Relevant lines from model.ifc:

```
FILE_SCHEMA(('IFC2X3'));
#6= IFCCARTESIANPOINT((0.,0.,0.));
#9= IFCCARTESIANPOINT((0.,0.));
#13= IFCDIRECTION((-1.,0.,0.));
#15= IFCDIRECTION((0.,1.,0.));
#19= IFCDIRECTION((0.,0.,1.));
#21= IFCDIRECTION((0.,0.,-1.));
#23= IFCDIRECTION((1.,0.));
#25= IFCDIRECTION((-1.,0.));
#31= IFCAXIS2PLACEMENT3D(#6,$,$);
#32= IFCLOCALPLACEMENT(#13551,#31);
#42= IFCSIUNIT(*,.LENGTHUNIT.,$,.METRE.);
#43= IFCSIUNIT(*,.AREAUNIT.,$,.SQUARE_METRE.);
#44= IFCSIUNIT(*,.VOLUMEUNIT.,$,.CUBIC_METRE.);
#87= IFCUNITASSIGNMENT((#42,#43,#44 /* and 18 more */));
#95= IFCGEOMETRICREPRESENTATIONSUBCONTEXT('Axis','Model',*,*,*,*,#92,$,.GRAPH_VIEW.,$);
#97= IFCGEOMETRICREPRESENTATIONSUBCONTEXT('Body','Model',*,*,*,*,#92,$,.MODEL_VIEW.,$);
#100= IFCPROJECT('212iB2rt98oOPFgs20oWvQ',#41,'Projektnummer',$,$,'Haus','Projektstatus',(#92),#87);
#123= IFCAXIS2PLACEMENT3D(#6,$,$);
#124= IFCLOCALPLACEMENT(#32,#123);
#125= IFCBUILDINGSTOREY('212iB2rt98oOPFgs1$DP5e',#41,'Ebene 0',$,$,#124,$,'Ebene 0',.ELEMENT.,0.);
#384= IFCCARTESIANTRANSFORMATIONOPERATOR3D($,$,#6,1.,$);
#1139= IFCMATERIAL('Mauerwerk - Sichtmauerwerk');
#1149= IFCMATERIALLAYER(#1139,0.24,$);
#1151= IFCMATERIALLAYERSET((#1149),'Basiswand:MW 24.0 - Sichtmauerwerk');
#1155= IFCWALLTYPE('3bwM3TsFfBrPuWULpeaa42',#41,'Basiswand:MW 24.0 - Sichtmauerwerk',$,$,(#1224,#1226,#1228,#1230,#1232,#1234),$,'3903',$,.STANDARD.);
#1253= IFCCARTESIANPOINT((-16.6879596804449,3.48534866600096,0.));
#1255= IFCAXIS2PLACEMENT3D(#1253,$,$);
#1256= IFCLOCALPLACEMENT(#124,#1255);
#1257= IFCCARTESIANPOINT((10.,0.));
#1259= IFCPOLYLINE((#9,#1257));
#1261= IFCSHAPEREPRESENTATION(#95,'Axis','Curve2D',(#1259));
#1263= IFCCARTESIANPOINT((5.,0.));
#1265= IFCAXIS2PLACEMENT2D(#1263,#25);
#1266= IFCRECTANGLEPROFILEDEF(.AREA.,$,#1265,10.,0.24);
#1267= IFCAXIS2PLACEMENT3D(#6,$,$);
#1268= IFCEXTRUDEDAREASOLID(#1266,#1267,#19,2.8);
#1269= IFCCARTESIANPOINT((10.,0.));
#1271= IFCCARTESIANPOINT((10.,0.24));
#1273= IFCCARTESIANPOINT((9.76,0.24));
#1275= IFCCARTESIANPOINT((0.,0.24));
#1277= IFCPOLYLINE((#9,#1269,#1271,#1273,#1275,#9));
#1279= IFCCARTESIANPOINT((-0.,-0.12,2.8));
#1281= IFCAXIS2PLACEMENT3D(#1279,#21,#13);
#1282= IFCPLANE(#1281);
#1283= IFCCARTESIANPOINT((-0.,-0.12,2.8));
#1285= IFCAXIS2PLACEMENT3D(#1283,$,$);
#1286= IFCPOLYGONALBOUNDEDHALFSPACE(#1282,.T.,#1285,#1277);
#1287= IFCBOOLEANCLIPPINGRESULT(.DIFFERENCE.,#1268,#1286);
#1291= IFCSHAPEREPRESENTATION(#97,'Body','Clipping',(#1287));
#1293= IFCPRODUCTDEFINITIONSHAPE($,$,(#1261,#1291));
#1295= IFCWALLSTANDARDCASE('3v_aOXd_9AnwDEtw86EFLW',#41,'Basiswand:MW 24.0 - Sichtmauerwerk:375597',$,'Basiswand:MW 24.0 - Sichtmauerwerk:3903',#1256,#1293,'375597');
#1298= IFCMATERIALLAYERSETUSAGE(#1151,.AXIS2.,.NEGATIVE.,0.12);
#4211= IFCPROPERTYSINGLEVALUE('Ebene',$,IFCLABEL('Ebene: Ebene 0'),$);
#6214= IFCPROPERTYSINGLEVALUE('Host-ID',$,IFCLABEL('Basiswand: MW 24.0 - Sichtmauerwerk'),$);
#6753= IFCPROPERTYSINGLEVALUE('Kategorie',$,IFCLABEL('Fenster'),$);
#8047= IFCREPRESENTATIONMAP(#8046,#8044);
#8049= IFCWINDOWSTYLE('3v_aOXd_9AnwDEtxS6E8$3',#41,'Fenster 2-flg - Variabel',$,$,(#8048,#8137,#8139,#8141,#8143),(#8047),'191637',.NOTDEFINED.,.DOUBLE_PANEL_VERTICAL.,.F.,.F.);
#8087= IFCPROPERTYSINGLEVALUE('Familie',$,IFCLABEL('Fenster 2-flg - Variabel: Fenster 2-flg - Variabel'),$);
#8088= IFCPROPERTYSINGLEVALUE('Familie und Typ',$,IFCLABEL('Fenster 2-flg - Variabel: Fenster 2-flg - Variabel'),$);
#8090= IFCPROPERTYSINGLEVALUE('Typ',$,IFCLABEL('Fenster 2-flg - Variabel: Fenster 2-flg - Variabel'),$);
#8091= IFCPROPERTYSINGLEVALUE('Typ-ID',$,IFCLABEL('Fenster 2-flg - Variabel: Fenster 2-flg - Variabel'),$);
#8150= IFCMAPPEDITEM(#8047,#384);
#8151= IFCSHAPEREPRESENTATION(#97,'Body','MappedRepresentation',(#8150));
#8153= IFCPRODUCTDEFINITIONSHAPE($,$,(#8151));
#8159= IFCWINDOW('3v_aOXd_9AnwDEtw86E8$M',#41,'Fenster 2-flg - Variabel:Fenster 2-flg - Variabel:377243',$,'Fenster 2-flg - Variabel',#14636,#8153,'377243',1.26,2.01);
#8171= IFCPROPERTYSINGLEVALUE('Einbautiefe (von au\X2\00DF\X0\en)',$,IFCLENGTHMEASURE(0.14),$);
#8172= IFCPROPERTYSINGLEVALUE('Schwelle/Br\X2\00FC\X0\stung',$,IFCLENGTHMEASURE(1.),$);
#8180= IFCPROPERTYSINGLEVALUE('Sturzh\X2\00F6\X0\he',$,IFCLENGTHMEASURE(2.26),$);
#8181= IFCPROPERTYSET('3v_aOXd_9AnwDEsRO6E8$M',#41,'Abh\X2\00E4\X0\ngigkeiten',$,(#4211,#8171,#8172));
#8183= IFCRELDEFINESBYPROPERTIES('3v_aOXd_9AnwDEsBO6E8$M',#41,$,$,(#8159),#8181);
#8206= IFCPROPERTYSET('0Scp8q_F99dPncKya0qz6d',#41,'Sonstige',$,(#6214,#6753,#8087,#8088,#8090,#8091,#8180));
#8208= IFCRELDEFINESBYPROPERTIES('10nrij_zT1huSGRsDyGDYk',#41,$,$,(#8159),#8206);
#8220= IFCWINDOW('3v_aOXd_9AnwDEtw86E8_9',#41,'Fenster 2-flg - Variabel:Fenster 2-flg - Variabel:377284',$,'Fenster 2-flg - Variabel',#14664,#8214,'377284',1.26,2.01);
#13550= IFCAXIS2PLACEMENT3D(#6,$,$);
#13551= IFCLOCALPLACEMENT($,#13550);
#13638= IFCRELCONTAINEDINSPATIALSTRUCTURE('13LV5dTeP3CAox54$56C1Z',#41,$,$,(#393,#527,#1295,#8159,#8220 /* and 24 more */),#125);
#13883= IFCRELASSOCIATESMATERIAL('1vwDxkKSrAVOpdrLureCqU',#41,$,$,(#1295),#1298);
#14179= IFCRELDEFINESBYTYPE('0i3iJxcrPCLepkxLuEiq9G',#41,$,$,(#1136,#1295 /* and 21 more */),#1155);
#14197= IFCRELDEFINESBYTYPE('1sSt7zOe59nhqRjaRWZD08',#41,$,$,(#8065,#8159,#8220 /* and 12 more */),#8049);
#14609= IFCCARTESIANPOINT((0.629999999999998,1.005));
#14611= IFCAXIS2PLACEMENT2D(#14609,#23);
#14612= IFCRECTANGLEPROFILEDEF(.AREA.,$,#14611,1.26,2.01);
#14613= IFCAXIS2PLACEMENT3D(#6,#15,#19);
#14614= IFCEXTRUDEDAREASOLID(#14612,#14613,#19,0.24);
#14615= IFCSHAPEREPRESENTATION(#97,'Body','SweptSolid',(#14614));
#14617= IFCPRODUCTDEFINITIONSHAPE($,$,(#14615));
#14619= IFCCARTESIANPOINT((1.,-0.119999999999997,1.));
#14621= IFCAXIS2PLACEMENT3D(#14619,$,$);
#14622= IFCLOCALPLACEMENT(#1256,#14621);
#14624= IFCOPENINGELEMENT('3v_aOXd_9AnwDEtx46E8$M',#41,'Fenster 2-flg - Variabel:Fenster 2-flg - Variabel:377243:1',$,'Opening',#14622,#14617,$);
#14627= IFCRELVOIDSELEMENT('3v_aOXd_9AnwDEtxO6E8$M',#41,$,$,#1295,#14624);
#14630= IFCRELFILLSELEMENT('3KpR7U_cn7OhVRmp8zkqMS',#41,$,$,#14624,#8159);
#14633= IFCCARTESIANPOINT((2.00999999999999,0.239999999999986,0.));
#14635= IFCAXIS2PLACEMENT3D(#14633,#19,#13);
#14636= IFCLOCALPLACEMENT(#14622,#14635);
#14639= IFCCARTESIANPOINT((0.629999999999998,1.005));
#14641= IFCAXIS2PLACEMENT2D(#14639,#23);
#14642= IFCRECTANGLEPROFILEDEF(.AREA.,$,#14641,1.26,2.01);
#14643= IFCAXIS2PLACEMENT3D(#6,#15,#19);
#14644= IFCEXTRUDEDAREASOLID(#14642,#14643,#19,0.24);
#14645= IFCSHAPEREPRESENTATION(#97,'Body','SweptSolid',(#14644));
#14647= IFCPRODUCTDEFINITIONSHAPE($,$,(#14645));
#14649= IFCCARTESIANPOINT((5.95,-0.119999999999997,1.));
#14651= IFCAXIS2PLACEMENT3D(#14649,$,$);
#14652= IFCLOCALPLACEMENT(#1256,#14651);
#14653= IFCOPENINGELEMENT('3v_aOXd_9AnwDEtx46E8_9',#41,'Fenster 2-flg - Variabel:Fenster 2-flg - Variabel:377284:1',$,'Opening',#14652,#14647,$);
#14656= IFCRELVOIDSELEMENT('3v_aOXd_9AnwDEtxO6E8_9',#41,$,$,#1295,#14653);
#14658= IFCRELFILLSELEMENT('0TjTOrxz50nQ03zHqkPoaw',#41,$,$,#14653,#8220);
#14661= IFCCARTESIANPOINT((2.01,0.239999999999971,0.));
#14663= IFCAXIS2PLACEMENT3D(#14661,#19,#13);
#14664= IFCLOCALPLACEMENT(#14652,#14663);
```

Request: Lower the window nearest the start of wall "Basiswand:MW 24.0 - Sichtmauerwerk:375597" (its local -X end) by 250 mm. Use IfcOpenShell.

```python
import numpy as np
import ifcopenshell
import ifcopenshell.api.geometry
import ifcopenshell.api.pset
import ifcopenshell.util.element
import ifcopenshell.util.placement
import ifcopenshell.util.unit

model = ifcopenshell.open("model.ifc")
unit_scale = ifcopenshell.util.unit.calculate_unit_scale(model)

window = model.by_guid("3v_aOXd_9AnwDEtw86E8$M")
opening = window.FillsVoids[0].RelatingOpeningElement
dz = -0.25 / unit_scale

shift = np.array([0.0, 0.0, dz])
# The window is placed relative to its opening, so it follows when the opening moves.
matrix = ifcopenshell.util.placement.get_local_placement(opening.ObjectPlacement)
matrix[:3, 3] += shift
ifcopenshell.api.geometry.edit_object_placement(
    model, product=opening, matrix=matrix, is_si=False, should_transform_children=True
)

# Keep the stored heights in step.
pset = model.by_id(ifcopenshell.util.element.get_pset(window, "Abhängigkeiten", should_inherit=False)["id"])
ifcopenshell.api.pset.edit_pset(model, pset=pset, properties={
    "Schwelle/Brüstung": model.create_entity("IfcLengthMeasure", ifcopenshell.util.element.get_pset(window, "Abhängigkeiten", "Schwelle/Brüstung") + dz),
})
pset = model.by_id(ifcopenshell.util.element.get_pset(window, "Sonstige", should_inherit=False)["id"])
ifcopenshell.api.pset.edit_pset(model, pset=pset, properties={
    "Sturzhöhe": model.create_entity("IfcLengthMeasure", ifcopenshell.util.element.get_pset(window, "Sonstige", "Sturzhöhe") + dz),
})

print(f"moved by {dz * unit_scale:+.3f} m")

model.write("model_rev.ifc")
```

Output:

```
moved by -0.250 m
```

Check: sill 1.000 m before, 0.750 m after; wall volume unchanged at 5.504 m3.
